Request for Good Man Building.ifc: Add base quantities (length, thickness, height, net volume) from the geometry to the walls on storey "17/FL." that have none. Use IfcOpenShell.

First a look at what the model holds.

```python
import ifcopenshell
import ifcopenshell.util.element
import ifcopenshell.util.unit

model = ifcopenshell.open("Good Man Building.ifc")
print(model.schema)
for unit_type in ("LENGTHUNIT", "AREAUNIT", "VOLUMEUNIT"):
    print(unit_type, ifcopenshell.util.unit.calculate_unit_scale(model, unit_type))
storey = next(s for s in model.by_type("IfcBuildingStorey") if s.Name == "17/FL.")
walls = [e for e in ifcopenshell.util.element.get_decomposition(storey) if e.is_a("IfcWall")]
for e in sorted(walls, key=lambda e: e.id()):
    print(e.id(), e.is_a(), e.Name, list(ifcopenshell.util.element.get_psets(e, qtos_only=True)), sep=" | ")
```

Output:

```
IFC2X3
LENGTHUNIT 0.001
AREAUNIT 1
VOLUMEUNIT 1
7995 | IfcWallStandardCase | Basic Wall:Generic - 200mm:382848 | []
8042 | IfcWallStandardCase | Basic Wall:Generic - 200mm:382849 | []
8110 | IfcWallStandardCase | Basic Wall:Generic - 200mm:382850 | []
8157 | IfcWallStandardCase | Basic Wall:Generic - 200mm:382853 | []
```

```python
import ifcopenshell
import ifcopenshell.api.pset
import ifcopenshell.geom
import ifcopenshell.util.element
import ifcopenshell.util.shape
import ifcopenshell.util.unit

model = ifcopenshell.open("Good Man Building.ifc")
unit_scale = ifcopenshell.util.unit.calculate_unit_scale(model)
volume_scale = ifcopenshell.util.unit.calculate_unit_scale(model, "VOLUMEUNIT")
settings = ifcopenshell.geom.settings()

storey = next(s for s in model.by_type("IfcBuildingStorey") if s.Name == "17/FL.")
walls = [e for e in ifcopenshell.util.element.get_decomposition(storey) if e.is_a("IfcWall")]

for e in sorted(walls, key=lambda e: e.id()):
    if ifcopenshell.util.element.get_psets(e, qtos_only=True, should_inherit=False):
        continue
    # Geometry comes back in metres, in the element's own axes.
    shape = ifcopenshell.geom.create_shape(settings, e)
    values = {
        "Length": ifcopenshell.util.shape.get_x(shape.geometry) / unit_scale,
        "Width": ifcopenshell.util.shape.get_y(shape.geometry) / unit_scale,
        "Height": ifcopenshell.util.shape.get_z(shape.geometry) / unit_scale,
        "NetVolume": ifcopenshell.util.shape.get_volume(shape.geometry) / volume_scale,
    }
    qto = ifcopenshell.api.pset.add_qto(model, product=e, name="BaseQuantities")
    ifcopenshell.api.pset.edit_qto(model, qto=qto, properties=values)
    print(e.id(), {k: round(v, 3) for k, v in values.items()})

model.write("Good Man Building_rev.ifc")
```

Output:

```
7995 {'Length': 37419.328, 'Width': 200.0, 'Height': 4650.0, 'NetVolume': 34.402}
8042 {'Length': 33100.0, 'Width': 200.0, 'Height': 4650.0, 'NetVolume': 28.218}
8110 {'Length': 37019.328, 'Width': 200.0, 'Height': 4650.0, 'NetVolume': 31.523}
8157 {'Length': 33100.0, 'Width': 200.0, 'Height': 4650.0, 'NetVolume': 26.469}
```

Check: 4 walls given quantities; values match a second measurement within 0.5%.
